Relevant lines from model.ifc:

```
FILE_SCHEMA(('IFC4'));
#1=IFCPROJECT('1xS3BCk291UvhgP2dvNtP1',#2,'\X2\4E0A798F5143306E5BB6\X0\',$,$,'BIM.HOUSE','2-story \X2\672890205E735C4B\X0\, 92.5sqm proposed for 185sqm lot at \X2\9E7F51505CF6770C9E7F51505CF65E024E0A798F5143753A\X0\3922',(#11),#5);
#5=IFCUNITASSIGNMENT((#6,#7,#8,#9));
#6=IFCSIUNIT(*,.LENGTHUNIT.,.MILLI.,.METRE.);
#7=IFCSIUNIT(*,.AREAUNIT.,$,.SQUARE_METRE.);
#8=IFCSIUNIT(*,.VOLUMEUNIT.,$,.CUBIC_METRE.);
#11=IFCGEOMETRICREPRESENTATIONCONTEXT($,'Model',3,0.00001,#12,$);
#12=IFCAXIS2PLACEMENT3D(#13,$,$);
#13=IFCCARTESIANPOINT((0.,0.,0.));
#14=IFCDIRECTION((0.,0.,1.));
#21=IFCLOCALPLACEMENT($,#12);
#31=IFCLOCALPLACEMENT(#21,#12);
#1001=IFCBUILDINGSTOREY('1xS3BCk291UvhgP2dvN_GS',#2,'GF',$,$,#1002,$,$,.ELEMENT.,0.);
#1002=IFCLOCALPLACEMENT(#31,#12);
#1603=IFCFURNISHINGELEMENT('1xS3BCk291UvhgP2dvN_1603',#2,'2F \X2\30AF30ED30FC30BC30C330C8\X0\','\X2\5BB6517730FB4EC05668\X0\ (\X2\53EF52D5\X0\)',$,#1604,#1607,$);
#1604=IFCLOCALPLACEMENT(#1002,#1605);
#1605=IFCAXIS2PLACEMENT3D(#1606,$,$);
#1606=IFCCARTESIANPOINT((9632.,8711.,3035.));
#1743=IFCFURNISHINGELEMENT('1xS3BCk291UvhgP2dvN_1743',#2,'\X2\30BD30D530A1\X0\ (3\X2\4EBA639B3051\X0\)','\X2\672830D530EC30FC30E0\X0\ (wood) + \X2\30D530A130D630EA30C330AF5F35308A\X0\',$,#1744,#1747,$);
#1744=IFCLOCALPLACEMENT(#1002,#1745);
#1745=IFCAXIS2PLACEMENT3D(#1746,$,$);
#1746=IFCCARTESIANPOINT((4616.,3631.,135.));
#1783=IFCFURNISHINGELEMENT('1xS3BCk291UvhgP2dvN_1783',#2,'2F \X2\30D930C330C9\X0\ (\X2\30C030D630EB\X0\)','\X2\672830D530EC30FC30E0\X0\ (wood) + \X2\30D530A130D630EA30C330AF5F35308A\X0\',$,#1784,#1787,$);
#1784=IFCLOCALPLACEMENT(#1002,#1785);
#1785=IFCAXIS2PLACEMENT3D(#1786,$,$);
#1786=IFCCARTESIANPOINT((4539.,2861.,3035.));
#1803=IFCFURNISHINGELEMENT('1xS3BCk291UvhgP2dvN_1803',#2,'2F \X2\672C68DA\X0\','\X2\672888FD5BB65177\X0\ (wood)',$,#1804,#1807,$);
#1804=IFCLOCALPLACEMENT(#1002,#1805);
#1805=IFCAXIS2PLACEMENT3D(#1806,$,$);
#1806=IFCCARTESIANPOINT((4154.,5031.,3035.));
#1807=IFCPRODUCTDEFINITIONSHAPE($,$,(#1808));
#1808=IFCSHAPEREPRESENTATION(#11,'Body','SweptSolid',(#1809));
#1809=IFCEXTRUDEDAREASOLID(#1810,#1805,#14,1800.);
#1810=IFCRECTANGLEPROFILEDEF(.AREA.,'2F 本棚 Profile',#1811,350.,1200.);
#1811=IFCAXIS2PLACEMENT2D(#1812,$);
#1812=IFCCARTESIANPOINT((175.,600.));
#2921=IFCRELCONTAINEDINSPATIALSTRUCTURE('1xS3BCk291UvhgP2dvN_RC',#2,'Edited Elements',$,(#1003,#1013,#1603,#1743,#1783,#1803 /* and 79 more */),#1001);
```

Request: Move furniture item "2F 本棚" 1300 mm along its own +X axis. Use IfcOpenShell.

```python
import ifcopenshell
import ifcopenshell.api.geometry
import ifcopenshell.util.placement

model = ifcopenshell.open("model.ifc")

item = model.by_guid("1xS3BCk291UvhgP2dvN_1803")
matrix = ifcopenshell.util.placement.get_local_placement(item.ObjectPlacement)
matrix[:3, 3] += matrix[:3, 0] * 1300.0
ifcopenshell.api.geometry.edit_object_placement(model, product=item, matrix=matrix, is_si=False)

print(ifcopenshell.util.placement.get_local_placement(item.ObjectPlacement).round(3) + 0.0)

model.write("model_edited.ifc")
```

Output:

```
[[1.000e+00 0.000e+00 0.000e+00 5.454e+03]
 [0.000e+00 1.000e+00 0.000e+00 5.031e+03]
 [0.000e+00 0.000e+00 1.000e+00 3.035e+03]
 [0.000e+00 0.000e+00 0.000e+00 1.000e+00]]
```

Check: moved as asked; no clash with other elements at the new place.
